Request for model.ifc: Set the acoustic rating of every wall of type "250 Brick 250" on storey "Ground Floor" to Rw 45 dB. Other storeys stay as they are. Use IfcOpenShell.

First a look at what the model holds.

```python
import ifcopenshell
import ifcopenshell.util.element

model = ifcopenshell.open("model.ifc")
print(model.schema)
storey = next(s for s in model.by_type("IfcBuildingStorey") if s.Name == "Ground Floor")
walls = [e for e in ifcopenshell.util.element.get_decomposition(storey) if e.is_a("IfcWall")]
seen = {}
for e in walls:
    element_type = ifcopenshell.util.element.get_type(e)
    key = (element_type.Name if element_type != e and element_type else None, ifcopenshell.util.element.get_pset(e, "Pset_WallCommon", "AcousticRating"))
    seen[key] = seen.get(key, 0) + 1
for (name, value), count in sorted(seen.items(), key=str):
    print(count, "x", name, "|", value)
```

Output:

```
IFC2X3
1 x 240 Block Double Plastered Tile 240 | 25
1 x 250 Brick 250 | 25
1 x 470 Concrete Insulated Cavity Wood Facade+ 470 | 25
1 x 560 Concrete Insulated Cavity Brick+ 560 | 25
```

```python
import ifcopenshell
import ifcopenshell.api.pset
import ifcopenshell.util.element

model = ifcopenshell.open("model.ifc")

storey = next(s for s in model.by_type("IfcBuildingStorey") if s.Name == "Ground Floor")
walls = [e for e in ifcopenshell.util.element.get_decomposition(storey) if e.is_a("IfcWall")]

count = 0
for e in walls:
    element_type = ifcopenshell.util.element.get_type(e)
    if element_type in (None, e) or element_type.Name != "250 Brick 250":
        continue
    # add_pset returns the element's existing set when there is one.
    pset = ifcopenshell.api.pset.add_pset(model, product=e, name="Pset_WallCommon")
    ifcopenshell.api.pset.edit_pset(model, pset=pset, properties={"AcousticRating": "Rw 45 dB"})
    count += 1

print(count, "walls updated")

model.write("model_updated.ifc")
```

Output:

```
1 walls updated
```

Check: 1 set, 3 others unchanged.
